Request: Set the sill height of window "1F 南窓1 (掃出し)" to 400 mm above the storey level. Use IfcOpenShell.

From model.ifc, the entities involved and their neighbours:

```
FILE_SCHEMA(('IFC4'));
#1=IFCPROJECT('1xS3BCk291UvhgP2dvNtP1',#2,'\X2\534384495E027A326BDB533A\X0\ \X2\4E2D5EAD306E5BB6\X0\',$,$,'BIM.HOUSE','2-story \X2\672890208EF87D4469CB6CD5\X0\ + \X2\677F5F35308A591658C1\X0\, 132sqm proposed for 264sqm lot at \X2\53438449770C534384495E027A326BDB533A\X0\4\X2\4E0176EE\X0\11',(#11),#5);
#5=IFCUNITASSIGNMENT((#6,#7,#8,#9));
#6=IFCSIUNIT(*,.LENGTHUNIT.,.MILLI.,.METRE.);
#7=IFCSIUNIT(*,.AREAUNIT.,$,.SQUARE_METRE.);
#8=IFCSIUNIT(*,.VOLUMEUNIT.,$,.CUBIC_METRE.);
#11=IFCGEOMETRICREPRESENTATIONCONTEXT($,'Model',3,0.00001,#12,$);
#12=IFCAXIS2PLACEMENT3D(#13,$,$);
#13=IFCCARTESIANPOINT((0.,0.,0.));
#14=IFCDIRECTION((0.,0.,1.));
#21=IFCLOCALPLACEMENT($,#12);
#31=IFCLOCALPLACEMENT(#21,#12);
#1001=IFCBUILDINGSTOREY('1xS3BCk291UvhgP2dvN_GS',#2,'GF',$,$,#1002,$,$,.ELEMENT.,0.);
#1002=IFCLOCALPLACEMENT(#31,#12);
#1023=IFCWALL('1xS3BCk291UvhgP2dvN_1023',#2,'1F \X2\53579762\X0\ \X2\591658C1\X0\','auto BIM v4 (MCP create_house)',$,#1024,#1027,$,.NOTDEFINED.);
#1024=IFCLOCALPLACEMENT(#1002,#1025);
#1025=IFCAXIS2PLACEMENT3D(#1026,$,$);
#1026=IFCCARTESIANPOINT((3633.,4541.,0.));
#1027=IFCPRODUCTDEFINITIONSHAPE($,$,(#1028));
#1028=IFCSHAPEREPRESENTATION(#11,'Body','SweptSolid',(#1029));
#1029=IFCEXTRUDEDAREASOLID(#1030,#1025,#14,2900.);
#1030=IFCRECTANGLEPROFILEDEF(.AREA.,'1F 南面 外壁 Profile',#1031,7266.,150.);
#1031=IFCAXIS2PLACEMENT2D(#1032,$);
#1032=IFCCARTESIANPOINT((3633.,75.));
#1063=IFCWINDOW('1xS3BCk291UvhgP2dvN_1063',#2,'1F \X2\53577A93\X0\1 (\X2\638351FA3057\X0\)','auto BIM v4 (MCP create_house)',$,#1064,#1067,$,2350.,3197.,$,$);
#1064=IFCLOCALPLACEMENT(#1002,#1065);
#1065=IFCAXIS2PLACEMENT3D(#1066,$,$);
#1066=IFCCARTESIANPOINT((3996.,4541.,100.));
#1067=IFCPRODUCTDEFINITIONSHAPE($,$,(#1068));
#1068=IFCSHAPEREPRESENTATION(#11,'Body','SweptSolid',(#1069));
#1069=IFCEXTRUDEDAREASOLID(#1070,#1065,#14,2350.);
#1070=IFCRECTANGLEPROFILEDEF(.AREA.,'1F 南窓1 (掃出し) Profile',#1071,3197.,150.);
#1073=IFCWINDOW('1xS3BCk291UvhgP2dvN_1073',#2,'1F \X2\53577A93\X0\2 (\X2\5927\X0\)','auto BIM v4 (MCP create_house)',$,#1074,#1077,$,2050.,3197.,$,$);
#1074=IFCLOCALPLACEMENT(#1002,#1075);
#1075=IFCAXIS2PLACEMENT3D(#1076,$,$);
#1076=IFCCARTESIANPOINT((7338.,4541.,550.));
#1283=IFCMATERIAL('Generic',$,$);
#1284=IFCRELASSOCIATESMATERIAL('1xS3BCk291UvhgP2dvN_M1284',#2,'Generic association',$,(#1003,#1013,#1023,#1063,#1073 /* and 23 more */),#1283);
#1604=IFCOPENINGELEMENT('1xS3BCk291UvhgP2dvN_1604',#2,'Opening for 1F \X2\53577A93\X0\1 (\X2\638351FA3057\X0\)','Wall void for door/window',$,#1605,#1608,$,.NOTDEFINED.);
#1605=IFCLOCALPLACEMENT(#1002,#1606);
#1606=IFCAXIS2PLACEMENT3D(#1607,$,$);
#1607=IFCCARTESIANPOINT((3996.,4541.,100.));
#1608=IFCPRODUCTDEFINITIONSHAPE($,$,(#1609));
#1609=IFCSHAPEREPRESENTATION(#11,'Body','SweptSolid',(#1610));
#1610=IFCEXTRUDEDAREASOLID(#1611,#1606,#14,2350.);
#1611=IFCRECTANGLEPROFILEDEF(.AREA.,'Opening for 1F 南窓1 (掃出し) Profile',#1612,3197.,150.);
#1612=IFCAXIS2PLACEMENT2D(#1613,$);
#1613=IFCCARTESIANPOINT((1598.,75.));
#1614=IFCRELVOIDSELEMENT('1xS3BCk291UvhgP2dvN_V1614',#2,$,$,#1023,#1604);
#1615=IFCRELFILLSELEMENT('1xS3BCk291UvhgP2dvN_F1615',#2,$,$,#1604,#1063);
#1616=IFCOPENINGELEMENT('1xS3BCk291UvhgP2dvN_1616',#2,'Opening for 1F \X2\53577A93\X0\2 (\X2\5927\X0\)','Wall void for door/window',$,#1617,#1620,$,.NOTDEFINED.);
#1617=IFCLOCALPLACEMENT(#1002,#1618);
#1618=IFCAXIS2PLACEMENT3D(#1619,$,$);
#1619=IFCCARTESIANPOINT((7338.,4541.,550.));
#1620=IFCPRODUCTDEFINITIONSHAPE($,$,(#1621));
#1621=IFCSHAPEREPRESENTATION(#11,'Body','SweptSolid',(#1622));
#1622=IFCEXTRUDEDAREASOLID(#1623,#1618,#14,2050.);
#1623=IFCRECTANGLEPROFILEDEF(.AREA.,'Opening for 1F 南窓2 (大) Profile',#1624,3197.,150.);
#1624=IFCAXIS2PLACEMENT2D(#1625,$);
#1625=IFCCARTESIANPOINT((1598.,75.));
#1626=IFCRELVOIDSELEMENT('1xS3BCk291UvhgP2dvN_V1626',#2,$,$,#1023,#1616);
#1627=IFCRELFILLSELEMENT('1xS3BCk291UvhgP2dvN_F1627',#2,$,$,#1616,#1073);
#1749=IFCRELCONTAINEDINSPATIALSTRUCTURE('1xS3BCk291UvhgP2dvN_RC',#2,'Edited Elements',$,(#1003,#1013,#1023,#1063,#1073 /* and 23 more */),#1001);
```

```python
import numpy as np
import ifcopenshell
import ifcopenshell.api.geometry
import ifcopenshell.geom
import ifcopenshell.util.element
import ifcopenshell.util.placement
import ifcopenshell.util.shape
import ifcopenshell.util.unit

model = ifcopenshell.open("model.ifc")
unit_scale = ifcopenshell.util.unit.calculate_unit_scale(model)

window = model.by_id(1063)
opening = window.FillsVoids[0].RelatingOpeningElement
storey = ifcopenshell.util.element.get_container(window, ifc_class="IfcBuildingStorey")
level = ifcopenshell.util.placement.get_local_placement(storey.ObjectPlacement)[2, 3]

# The opening's origin need not be at the sill, so measure its lowest point.
shape = ifcopenshell.geom.create_shape(ifcopenshell.geom.settings(), opening)
bottom = ifcopenshell.util.shape.get_shape_bottom_elevation(shape, shape.geometry) / unit_scale
dz = level + 400.0 - bottom

shift = np.array([0.0, 0.0, dz])
# The window is not placed relative to its opening, so move both.
for product in (opening, window):
    matrix = ifcopenshell.util.placement.get_local_placement(product.ObjectPlacement)
    matrix[:3, 3] += shift
    ifcopenshell.api.geometry.edit_object_placement(model, product=product, matrix=matrix, is_si=False)

print(f"moved by {dz * unit_scale:+.3f} m")

model.write("model_edited.ifc")
```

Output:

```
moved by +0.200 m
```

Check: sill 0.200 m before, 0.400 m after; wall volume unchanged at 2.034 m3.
